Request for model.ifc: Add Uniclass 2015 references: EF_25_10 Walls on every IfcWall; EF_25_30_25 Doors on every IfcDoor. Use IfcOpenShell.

First a look at what the model holds.

```python
import ifcopenshell

model = ifcopenshell.open("model.ifc")
print(model.schema)
print("classifications:", [c.Name for c in model.by_type("IfcClassification")])
for ifc_class in ("IfcDoor", "IfcRoof", "IfcStair", "IfcWall", "IfcWindow"):
    print(ifc_class, len(model.by_type(ifc_class)))
```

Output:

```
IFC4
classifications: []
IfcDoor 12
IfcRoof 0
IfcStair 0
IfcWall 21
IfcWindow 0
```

```python
import ifcopenshell
import ifcopenshell.api.classification

model = ifcopenshell.open("model.ifc")

system = ifcopenshell.api.classification.add_classification(model, classification="Uniclass 2015")

codes = {
    "IfcWall": ("EF_25_10", "Walls"),
    "IfcDoor": ("EF_25_30_25", "Doors"),
}
for ifc_class, (code, name) in codes.items():
    products = model.by_type(ifc_class)
    ifcopenshell.api.classification.add_reference(
        model, products=products, classification=system, identification=code, name=name
    )
    print(code, len(products))

model.write("model-out.ifc")
```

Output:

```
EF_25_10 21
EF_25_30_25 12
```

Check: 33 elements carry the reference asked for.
